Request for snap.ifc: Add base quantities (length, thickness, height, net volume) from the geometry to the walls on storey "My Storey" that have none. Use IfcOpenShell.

First a look at what the model holds.

```python
import ifcopenshell
import ifcopenshell.util.element
import ifcopenshell.util.unit

model = ifcopenshell.open("snap.ifc")
print(model.schema)
for unit_type in ("LENGTHUNIT", "AREAUNIT", "VOLUMEUNIT"):
    print(unit_type, ifcopenshell.util.unit.calculate_unit_scale(model, unit_type))
storey = next(s for s in model.by_type("IfcBuildingStorey") if s.Name == "My Storey")
walls = [e for e in ifcopenshell.util.element.get_decomposition(storey) if e.is_a("IfcWall")]
for e in sorted(walls, key=lambda e: e.id()):
    print(e.id(), e.is_a(), e.Name, list(ifcopenshell.util.element.get_psets(e, qtos_only=True)), sep=" | ")
```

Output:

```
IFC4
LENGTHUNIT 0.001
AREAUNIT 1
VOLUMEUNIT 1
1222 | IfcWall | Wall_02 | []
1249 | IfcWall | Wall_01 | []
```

```python
import ifcopenshell
import ifcopenshell.api.pset
import ifcopenshell.geom
import ifcopenshell.util.element
import ifcopenshell.util.shape
import ifcopenshell.util.unit

model = ifcopenshell.open("snap.ifc")
unit_scale = ifcopenshell.util.unit.calculate_unit_scale(model)
volume_scale = ifcopenshell.util.unit.calculate_unit_scale(model, "VOLUMEUNIT")
settings = ifcopenshell.geom.settings()

storey = next(s for s in model.by_type("IfcBuildingStorey") if s.Name == "My Storey")
walls = [e for e in ifcopenshell.util.element.get_decomposition(storey) if e.is_a("IfcWall")]

for e in sorted(walls, key=lambda e: e.id()):
    if ifcopenshell.util.element.get_psets(e, qtos_only=True, should_inherit=False):
        continue
    # Geometry comes back in metres, in the element's own axes.
    shape = ifcopenshell.geom.create_shape(settings, e)
    values = {
        "Length": ifcopenshell.util.shape.get_x(shape.geometry) / unit_scale,
        "Width": ifcopenshell.util.shape.get_y(shape.geometry) / unit_scale,
        "Height": ifcopenshell.util.shape.get_z(shape.geometry) / unit_scale,
        "NetVolume": ifcopenshell.util.shape.get_volume(shape.geometry) / volume_scale,
    }
    qto = ifcopenshell.api.pset.add_qto(model, product=e, name="Qto_WallBaseQuantities")
    ifcopenshell.api.pset.edit_qto(model, qto=qto, properties=values)
    print(e.id(), {k: round(v, 3) for k, v in values.items()})

model.write("snap-out.ifc")
```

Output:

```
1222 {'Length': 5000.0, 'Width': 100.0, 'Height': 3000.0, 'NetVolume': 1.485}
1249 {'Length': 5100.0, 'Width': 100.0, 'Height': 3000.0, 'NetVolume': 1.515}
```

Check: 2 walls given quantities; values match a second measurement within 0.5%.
